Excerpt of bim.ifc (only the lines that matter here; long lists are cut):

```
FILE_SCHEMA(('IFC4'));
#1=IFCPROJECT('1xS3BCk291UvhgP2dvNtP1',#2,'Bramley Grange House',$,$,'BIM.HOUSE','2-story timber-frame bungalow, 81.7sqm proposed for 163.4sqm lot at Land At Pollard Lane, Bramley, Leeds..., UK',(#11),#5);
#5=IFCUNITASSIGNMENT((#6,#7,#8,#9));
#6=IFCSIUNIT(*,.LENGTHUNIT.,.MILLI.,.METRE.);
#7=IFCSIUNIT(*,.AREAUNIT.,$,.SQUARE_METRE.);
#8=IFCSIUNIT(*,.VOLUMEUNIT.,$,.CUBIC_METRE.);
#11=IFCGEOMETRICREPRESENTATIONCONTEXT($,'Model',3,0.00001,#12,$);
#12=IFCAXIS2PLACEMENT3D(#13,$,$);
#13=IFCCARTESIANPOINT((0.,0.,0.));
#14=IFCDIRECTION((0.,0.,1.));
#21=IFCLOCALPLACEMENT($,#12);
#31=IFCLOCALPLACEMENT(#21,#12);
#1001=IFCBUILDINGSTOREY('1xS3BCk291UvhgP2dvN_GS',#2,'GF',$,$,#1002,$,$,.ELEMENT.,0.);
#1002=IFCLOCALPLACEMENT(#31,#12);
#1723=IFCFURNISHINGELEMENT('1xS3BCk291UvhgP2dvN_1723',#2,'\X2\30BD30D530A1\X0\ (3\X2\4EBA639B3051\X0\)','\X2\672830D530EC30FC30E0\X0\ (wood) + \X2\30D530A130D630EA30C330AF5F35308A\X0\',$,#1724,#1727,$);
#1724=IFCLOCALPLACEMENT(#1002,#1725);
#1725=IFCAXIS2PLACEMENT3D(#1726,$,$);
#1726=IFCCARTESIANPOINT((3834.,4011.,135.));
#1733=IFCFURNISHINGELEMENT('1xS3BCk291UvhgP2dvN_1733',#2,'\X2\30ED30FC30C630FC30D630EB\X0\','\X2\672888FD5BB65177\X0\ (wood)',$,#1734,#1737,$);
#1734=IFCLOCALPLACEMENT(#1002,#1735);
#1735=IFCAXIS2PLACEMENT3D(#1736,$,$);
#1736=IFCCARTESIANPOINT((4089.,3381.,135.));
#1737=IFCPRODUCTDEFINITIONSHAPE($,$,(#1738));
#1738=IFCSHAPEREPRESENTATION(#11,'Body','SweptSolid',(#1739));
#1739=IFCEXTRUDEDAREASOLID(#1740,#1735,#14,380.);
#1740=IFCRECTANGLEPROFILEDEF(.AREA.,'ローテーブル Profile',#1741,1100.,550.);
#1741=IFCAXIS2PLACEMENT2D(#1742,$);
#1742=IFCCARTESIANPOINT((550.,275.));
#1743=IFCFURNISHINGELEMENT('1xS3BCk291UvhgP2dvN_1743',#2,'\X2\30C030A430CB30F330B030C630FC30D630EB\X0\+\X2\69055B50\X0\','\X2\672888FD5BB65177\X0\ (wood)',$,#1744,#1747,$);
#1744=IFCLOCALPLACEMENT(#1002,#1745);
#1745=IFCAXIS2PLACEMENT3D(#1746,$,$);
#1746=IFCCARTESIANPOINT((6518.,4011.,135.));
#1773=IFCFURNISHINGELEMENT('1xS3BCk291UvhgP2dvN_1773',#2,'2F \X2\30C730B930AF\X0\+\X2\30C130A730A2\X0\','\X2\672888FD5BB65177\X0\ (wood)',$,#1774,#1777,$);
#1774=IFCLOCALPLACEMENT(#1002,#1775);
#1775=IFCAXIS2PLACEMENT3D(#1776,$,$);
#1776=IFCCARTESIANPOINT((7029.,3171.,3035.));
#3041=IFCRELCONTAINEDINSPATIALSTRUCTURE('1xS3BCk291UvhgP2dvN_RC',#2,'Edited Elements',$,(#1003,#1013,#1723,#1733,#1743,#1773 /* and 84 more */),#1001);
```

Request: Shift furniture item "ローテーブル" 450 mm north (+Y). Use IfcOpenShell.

```python
import ifcopenshell
import ifcopenshell.api.geometry
import ifcopenshell.util.placement
import ifcopenshell.util.unit

model = ifcopenshell.open("bim.ifc")
unit_scale = ifcopenshell.util.unit.calculate_unit_scale(model)

item = model.by_id(1733)
matrix = ifcopenshell.util.placement.get_local_placement(item.ObjectPlacement)
matrix[1, 3] += 0.45 / unit_scale
ifcopenshell.api.geometry.edit_object_placement(model, product=item, matrix=matrix, is_si=False)

print(ifcopenshell.util.placement.get_local_placement(item.ObjectPlacement).round(3) + 0.0)

model.write("bim_edited.ifc")
```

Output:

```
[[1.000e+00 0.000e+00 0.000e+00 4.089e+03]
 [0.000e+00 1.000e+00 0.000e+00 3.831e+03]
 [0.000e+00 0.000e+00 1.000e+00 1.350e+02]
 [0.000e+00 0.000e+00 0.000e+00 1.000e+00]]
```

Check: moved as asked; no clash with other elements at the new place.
